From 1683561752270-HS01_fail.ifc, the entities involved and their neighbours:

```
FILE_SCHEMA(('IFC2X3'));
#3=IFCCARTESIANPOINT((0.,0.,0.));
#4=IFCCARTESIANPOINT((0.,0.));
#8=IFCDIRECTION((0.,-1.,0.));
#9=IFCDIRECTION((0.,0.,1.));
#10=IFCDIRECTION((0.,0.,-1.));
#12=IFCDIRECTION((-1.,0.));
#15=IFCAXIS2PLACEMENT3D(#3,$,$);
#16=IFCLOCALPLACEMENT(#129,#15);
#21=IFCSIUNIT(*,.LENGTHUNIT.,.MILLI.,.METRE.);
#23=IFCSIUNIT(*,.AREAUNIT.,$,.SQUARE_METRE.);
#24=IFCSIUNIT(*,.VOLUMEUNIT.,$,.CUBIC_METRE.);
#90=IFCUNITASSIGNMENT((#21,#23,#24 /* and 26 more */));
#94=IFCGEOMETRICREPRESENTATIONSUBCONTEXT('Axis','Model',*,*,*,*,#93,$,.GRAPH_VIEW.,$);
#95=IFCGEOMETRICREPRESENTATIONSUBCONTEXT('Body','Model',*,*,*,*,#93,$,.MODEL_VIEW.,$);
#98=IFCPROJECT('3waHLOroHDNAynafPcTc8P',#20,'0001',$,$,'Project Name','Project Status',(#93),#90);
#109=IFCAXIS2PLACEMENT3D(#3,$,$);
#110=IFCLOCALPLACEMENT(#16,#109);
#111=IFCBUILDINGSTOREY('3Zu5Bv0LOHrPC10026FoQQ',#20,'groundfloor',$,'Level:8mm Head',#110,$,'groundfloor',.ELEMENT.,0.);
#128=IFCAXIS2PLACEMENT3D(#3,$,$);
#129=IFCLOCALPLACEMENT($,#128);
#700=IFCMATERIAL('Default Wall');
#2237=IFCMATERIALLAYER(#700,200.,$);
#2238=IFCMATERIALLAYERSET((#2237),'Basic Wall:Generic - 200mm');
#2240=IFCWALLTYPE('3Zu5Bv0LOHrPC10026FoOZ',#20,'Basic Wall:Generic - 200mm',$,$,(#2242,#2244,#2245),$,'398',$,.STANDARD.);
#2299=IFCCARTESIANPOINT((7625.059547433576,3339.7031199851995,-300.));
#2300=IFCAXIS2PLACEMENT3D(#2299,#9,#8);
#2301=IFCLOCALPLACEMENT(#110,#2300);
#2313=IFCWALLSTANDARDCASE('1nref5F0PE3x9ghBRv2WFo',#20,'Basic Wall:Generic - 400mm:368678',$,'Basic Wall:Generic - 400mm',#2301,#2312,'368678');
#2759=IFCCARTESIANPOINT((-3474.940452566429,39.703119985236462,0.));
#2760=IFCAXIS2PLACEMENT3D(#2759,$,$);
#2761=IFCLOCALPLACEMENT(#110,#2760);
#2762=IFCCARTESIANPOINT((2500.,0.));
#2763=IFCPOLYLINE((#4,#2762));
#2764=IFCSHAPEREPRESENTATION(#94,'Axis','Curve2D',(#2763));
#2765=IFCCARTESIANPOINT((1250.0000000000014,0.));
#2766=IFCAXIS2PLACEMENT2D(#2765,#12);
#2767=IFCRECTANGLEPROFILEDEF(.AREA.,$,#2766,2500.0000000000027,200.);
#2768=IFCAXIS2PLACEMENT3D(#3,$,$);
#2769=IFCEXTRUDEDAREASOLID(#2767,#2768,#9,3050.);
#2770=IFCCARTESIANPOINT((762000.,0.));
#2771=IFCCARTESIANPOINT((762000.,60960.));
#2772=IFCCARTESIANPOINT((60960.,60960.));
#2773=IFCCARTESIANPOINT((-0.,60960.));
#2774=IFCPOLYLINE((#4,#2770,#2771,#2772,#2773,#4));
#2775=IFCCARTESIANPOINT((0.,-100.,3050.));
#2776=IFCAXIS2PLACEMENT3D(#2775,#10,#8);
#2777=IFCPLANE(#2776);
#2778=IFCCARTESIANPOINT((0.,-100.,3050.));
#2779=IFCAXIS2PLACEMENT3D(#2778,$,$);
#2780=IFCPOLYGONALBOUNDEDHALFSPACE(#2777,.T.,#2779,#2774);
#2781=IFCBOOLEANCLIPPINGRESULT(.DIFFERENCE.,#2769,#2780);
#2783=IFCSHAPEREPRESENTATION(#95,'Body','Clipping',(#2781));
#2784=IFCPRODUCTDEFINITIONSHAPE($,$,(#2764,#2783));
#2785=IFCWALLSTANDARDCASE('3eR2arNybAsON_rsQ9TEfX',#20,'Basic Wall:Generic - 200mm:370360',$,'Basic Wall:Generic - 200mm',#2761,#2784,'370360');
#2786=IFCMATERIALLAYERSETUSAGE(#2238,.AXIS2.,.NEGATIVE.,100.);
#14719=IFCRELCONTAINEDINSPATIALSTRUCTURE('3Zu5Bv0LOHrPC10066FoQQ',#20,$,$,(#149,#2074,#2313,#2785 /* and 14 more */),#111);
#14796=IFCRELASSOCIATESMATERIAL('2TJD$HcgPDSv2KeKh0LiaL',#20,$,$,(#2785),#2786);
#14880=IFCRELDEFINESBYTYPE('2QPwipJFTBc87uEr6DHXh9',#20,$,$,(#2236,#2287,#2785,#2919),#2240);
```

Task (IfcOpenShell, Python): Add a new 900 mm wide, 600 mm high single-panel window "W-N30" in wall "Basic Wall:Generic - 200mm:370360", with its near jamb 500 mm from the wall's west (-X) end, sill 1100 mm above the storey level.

```python
import numpy as np
import ifcopenshell
import ifcopenshell.api.feature
import ifcopenshell.api.geometry
import ifcopenshell.api.root
import ifcopenshell.api.spatial
import ifcopenshell.api.type
import ifcopenshell.geom
import ifcopenshell.util.element
import ifcopenshell.util.placement
import ifcopenshell.util.representation
import ifcopenshell.util.shape
import ifcopenshell.util.unit

model = ifcopenshell.open("1683561752270-HS01_fail.ifc")
unit_scale = ifcopenshell.util.unit.calculate_unit_scale(model)
settings = ifcopenshell.geom.settings()


def volume(element):
    """Net volume in cubic metres, openings subtracted."""
    shape = ifcopenshell.geom.create_shape(settings, element)
    return ifcopenshell.util.shape.get_volume(shape.geometry)


wall = model.by_guid("3eR2arNybAsON_rsQ9TEfX")
storey = ifcopenshell.util.element.get_container(wall, ifc_class="IfcBuildingStorey")
context = ifcopenshell.util.representation.get_context(model, "Model", "Body", "MODEL_VIEW")
before = volume(wall)

width, height, from_end, sill = 0.9, 0.6, 0.5, 1.1  # metres

# The wall runs along its own X axis, and the end named is its -X end.
wall_shape = ifcopenshell.geom.create_shape(settings, wall)
x, y, z = ifcopenshell.util.shape.get_vertices(wall_shape.geometry).T
start = x.min() + from_end
face, thickness = float(y.min()), float(y.max() - y.min())
wall_matrix = ifcopenshell.util.placement.get_local_placement(wall.ObjectPlacement)
level = ifcopenshell.util.placement.get_local_placement(storey.ObjectPlacement)[2, 3]


def in_wall(x, y):
    """Placement at x, y metres in the wall's axes, at sill height."""
    matrix = wall_matrix.copy()
    matrix[:, 3] = wall_matrix @ np.array([x / unit_scale, y / unit_scale, 0.0, 1.0])
    matrix[2, 3] = level + sill / unit_scale
    return matrix


# Opening: a box that overshoots both wall faces by 50 mm.
opening = ifcopenshell.api.root.create_entity(model, ifc_class="IfcOpeningElement")
box = ifcopenshell.api.geometry.add_wall_representation(
    model, context=context, length=width, height=height, thickness=thickness + 0.1
)
ifcopenshell.api.geometry.assign_representation(model, product=opening, representation=box)
ifcopenshell.api.geometry.edit_object_placement(model, product=opening, matrix=in_wall(start, face - 0.05), is_si=False)
ifcopenshell.api.feature.add_feature(model, feature=opening, element=wall)

window = ifcopenshell.api.root.create_entity(model, ifc_class="IfcWindow", name="W-N30")
window.OverallWidth, window.OverallHeight = width / unit_scale, height / unit_scale
body = ifcopenshell.api.geometry.add_window_representation(
    model,
    context=context,
    overall_width=window.OverallWidth,
    overall_height=window.OverallHeight,
    partition_type="SINGLE_PANEL",
)
ifcopenshell.api.geometry.assign_representation(model, product=window, representation=body)
ifcopenshell.api.spatial.assign_container(model, products=[window], relating_structure=storey)
fills = ifcopenshell.api.feature.add_filling(model, opening=opening, element=window)
fills.OwnerHistory = window.OwnerHistory  # required in IFC2X3

# IFC2X3 keeps the operation on the window style.
style = ifcopenshell.api.root.create_entity(model, ifc_class="IfcWindowStyle", name="W-N30")
style.OperationType, style.ConstructionType = "SINGLE_PANEL", "NOTDEFINED"
style.ParameterTakesPrecedence = style.Sizeable = False
ifcopenshell.api.type.assign_type(model, related_objects=[window], relating_type=style)

# Centre the window in the wall's thickness.
ifcopenshell.api.geometry.edit_object_placement(model, product=window, matrix=in_wall(start, face), is_si=False)
window_shape = ifcopenshell.geom.create_shape(settings, window)
depth = ifcopenshell.util.shape.get_vertices(window_shape.geometry)[:, 1]
offset = face + thickness / 2 - (depth.min() + depth.max()) / 2
ifcopenshell.api.geometry.edit_object_placement(model, product=window, matrix=in_wall(start, offset), is_si=False)

after = volume(wall)

print(f"wall volume {before:.3f} -> {after:.3f} m3")

model.write("1683561752270-HS01_fail_v2.ifc")
```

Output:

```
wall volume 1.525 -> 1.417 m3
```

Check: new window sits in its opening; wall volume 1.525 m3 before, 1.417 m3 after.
